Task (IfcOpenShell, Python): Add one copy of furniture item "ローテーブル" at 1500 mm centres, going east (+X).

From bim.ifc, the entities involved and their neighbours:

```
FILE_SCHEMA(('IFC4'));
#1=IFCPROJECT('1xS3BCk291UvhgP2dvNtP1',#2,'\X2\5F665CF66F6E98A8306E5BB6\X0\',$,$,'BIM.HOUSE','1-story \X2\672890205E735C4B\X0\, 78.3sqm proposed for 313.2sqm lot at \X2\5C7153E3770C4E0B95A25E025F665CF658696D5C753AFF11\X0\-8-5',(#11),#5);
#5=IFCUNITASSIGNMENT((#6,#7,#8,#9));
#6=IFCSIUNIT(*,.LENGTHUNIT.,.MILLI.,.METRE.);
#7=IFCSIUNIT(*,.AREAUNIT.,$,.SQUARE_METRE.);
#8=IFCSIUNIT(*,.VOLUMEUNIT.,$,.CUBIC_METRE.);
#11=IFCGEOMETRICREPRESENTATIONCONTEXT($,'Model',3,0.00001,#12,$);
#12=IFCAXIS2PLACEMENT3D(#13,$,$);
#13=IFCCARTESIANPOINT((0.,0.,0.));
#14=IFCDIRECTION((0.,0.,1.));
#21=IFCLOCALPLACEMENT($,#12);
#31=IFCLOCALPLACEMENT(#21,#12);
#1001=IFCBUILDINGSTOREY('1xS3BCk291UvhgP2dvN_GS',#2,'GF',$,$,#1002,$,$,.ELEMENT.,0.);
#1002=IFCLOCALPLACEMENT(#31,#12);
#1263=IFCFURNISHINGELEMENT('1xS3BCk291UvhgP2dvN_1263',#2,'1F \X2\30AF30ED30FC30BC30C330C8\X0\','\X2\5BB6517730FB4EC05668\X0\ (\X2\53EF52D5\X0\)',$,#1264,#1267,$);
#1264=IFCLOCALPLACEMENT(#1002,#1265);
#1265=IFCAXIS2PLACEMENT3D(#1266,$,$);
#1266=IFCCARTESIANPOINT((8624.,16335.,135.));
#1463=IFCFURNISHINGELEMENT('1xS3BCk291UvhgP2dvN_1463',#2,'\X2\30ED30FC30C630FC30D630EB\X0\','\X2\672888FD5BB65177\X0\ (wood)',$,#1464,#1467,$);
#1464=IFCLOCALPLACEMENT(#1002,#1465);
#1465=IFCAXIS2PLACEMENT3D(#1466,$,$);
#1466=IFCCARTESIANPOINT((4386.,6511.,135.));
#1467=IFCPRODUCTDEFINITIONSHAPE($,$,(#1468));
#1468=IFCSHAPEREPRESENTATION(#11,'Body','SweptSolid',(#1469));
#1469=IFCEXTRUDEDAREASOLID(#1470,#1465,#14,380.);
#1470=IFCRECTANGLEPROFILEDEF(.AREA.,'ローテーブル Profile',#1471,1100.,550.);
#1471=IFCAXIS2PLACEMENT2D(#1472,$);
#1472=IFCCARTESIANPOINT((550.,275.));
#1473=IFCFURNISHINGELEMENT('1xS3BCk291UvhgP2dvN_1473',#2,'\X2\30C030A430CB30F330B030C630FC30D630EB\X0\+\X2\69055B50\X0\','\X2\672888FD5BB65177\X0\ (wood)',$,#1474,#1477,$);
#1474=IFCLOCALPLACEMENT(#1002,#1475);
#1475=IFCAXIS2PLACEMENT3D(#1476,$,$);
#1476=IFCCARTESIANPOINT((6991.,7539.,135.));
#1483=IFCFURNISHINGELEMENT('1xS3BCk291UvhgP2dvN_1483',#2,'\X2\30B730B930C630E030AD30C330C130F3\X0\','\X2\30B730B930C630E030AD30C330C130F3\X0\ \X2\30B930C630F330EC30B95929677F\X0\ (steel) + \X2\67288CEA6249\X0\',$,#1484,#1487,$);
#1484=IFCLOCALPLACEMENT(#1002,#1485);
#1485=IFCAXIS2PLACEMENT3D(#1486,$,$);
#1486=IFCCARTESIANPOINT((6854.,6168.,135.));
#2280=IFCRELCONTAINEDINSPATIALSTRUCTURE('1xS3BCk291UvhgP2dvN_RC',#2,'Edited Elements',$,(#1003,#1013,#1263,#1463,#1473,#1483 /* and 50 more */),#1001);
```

```python
import numpy as np
import ifcopenshell
import ifcopenshell.api.geometry
import ifcopenshell.api.root
import ifcopenshell.util.element
import ifcopenshell.util.placement

model = ifcopenshell.open("bim.ifc")


def reuse_history(source, copy):
    """copy_class also copies each property set's owner history, people and application; keep the originals."""
    for rel in copy.IsDefinedBy:
        if rel.is_a("IfcRelDefinesByProperties") and (history := rel.RelatingPropertyDefinition.OwnerHistory):
            rel.RelatingPropertyDefinition.OwnerHistory = source.OwnerHistory
            ifcopenshell.util.element.remove_deep2(model, history)


source = model.by_guid("1xS3BCk291UvhgP2dvN_1463")
base = ifcopenshell.util.placement.get_local_placement(source.ObjectPlacement)
step = np.array([1.0, 0.0, 0.0]) * 1500.0

for i in range(1, 2):
    copy = ifcopenshell.api.root.copy_class(model, product=source)
    copy.Representation = ifcopenshell.util.element.copy_deep(
        model, source.Representation, exclude=["IfcGeometricRepresentationContext", "IfcRepresentationMap"]
    )
    reuse_history(source, copy)
    matrix = base.copy()
    matrix[:3, 3] += i * step
    print("added at", matrix[:3, 3].round(3) + 0.0)
    ifcopenshell.api.geometry.edit_object_placement(model, product=copy, matrix=matrix, is_si=False)

model.write("bim_updated.ifc")
```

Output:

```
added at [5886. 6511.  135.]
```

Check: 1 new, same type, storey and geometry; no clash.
